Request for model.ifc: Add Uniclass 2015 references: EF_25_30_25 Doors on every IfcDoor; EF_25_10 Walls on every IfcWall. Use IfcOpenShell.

First a look at what the model holds.

```python
import ifcopenshell

model = ifcopenshell.open("model.ifc")
print(model.schema)
print("classifications:", [c.Name for c in model.by_type("IfcClassification")])
for ifc_class in ("IfcDoor", "IfcRoof", "IfcStair", "IfcWall", "IfcWindow"):
    print(ifc_class, len(model.by_type(ifc_class)))
```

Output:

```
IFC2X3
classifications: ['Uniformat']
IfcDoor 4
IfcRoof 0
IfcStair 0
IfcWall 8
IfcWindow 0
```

```python
import ifcopenshell
import ifcopenshell.api.classification

model = ifcopenshell.open("model.ifc")

# IFC2X3 requires Source and Edition and has no link from the project to the system.
system = model.create_entity("IfcClassification", Source="NBS", Edition="2015", Name="Uniclass 2015")

codes = {
    "IfcDoor": ("EF_25_30_25", "Doors"),
    "IfcWall": ("EF_25_10", "Walls"),
}
for ifc_class, (code, name) in codes.items():
    products = model.by_type(ifc_class)
    ifcopenshell.api.classification.add_reference(
        model, products=products, classification=system, identification=code, name=name
    )
    print(code, len(products))

model.write("model-out.ifc")
```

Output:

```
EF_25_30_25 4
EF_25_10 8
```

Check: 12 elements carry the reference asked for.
